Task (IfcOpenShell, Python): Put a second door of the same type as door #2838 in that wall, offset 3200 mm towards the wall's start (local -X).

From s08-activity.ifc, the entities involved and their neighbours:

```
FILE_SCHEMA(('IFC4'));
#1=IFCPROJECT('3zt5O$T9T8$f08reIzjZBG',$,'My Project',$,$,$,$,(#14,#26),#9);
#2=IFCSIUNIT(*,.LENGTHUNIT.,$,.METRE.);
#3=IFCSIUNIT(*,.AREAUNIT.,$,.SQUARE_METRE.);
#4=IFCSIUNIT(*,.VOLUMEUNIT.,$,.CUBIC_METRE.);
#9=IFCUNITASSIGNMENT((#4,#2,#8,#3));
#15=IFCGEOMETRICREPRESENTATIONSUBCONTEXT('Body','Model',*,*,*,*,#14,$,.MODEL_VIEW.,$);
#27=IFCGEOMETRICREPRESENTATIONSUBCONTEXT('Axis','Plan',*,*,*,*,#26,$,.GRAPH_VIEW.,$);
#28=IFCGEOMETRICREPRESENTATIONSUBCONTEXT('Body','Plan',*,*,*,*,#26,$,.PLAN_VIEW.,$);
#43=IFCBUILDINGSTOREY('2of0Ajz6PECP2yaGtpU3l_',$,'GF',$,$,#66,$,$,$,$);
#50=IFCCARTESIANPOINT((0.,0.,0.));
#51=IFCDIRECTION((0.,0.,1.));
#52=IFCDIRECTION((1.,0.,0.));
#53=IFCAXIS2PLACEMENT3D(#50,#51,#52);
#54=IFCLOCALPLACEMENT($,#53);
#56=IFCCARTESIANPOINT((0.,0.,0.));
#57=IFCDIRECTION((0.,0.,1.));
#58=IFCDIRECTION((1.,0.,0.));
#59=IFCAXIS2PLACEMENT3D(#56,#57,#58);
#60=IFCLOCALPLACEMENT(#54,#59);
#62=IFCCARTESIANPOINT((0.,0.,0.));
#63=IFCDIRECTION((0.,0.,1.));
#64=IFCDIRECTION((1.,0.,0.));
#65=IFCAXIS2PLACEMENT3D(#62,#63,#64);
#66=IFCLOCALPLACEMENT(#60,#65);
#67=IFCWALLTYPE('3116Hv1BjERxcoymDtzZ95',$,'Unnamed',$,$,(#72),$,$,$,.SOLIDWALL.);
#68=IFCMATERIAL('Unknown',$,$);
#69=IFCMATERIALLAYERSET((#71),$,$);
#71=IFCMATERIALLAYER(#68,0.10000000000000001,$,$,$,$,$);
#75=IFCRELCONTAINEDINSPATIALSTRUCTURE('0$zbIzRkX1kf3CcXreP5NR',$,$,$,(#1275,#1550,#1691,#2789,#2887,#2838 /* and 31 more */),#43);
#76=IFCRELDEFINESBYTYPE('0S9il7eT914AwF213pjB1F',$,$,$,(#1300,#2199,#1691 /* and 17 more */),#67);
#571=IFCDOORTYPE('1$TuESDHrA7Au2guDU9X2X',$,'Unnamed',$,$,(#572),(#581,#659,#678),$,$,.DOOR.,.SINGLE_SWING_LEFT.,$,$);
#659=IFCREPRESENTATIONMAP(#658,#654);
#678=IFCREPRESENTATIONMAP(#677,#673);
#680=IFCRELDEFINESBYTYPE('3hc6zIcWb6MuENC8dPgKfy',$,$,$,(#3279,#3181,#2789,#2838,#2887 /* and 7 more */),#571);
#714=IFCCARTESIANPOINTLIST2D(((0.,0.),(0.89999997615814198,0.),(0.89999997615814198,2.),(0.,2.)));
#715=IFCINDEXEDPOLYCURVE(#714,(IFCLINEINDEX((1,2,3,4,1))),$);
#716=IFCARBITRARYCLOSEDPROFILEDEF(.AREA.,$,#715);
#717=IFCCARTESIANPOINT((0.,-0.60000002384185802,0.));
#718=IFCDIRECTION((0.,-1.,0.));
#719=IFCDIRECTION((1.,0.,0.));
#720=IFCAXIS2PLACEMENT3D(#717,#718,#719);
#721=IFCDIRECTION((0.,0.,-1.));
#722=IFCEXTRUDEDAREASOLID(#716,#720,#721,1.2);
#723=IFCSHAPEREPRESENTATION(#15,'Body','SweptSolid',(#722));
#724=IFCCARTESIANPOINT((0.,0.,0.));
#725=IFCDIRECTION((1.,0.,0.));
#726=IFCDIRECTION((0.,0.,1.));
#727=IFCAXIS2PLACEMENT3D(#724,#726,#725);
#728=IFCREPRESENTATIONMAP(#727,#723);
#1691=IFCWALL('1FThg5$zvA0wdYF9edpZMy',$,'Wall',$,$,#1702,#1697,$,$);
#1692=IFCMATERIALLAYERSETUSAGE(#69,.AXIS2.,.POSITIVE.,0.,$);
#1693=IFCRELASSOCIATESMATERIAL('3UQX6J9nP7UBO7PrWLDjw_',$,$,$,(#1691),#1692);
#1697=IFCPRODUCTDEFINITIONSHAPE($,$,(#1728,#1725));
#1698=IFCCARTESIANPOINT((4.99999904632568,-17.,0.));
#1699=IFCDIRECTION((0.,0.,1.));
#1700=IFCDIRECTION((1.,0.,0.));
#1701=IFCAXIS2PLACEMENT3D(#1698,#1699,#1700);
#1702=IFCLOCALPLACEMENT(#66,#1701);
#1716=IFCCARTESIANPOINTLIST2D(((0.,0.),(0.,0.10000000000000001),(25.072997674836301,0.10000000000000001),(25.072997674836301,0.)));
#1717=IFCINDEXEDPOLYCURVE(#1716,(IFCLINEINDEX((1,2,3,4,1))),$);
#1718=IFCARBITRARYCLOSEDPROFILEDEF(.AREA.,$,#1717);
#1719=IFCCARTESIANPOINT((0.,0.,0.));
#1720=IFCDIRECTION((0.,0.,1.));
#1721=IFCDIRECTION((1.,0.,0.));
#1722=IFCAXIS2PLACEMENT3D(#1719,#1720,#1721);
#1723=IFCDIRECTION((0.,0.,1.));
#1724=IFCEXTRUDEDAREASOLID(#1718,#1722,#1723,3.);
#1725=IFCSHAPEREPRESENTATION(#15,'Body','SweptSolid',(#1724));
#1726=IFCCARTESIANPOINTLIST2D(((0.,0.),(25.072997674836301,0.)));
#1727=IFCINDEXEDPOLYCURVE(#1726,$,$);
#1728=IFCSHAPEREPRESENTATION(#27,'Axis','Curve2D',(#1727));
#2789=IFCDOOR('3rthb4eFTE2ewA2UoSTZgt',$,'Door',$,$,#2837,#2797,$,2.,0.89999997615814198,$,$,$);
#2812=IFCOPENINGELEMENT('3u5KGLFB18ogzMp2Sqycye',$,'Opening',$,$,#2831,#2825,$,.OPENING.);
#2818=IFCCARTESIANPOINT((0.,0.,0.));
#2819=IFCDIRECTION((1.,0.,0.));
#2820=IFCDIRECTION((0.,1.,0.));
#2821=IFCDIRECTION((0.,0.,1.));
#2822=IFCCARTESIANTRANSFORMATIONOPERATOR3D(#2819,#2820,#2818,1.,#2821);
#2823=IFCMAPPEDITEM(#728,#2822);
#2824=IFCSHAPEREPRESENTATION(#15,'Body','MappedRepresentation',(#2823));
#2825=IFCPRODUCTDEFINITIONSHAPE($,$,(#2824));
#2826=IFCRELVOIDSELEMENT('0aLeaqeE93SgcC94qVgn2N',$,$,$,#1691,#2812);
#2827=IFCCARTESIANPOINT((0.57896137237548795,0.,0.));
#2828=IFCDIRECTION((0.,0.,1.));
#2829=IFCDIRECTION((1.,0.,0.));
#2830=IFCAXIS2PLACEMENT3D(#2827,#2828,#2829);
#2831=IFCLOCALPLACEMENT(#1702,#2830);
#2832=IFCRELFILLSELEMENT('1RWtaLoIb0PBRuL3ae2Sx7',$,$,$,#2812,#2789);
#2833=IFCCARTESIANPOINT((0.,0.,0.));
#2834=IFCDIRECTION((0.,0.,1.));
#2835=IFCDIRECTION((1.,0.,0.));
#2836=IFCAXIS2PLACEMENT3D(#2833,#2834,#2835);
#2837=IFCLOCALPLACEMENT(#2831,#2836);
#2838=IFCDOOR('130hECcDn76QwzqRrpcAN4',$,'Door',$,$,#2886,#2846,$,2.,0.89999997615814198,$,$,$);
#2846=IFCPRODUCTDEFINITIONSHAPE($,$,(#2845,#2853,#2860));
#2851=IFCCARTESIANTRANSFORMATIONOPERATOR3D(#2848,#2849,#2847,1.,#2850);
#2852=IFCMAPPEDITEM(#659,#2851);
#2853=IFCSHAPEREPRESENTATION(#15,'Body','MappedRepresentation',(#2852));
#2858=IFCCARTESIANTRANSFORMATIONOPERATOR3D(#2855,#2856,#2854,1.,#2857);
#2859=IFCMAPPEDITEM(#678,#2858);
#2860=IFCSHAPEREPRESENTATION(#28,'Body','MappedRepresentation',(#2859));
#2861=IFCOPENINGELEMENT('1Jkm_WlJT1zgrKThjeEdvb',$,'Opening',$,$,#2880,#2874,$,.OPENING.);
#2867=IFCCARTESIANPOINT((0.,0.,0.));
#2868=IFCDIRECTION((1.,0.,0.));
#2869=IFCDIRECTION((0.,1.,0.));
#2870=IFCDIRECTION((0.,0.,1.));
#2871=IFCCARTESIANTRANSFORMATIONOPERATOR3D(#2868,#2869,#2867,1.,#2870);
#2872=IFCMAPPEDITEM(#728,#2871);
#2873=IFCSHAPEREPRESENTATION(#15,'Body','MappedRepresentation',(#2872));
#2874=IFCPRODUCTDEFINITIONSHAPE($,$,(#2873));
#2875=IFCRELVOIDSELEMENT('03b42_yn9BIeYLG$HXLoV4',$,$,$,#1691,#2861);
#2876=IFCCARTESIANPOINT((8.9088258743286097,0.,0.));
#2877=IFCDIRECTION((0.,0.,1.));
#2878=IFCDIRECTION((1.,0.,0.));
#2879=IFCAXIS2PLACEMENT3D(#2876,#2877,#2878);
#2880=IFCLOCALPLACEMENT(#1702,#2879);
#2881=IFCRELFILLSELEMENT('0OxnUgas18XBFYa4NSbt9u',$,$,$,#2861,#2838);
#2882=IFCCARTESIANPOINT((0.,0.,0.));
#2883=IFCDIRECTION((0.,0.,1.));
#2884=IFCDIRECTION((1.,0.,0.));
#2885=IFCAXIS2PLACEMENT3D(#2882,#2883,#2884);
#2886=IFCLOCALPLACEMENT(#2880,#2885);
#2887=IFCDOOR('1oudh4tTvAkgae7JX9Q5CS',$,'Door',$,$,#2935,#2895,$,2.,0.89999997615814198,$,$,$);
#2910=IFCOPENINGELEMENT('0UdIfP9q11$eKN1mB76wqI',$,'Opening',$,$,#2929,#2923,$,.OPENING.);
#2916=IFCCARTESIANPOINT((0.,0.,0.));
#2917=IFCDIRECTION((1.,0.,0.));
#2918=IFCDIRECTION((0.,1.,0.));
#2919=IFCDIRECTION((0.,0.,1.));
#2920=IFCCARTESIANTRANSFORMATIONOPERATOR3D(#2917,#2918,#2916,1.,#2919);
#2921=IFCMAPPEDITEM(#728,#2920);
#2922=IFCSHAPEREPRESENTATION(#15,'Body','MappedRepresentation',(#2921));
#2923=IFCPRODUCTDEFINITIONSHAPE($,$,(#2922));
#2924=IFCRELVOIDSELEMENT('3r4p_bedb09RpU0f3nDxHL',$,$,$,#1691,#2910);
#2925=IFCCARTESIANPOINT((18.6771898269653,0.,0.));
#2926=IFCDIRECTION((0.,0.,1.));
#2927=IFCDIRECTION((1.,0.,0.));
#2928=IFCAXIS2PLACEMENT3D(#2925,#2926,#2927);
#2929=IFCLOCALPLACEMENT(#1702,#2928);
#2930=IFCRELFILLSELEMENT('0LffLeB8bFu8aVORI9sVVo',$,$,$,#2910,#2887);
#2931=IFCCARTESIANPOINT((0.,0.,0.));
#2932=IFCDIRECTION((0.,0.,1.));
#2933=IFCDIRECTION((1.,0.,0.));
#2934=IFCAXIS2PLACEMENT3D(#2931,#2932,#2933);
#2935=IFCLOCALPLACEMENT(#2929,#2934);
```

```python
import ifcopenshell
import ifcopenshell.api.feature
import ifcopenshell.api.geometry
import ifcopenshell.api.root
import ifcopenshell.geom
import ifcopenshell.util.element
import ifcopenshell.util.placement
import ifcopenshell.util.shape
import ifcopenshell.util.unit

model = ifcopenshell.open("s08-activity.ifc")
unit_scale = ifcopenshell.util.unit.calculate_unit_scale(model)
settings = ifcopenshell.geom.settings()


def volume(element):
    """Net volume in cubic metres, openings subtracted."""
    shape = ifcopenshell.geom.create_shape(settings, element)
    return ifcopenshell.util.shape.get_volume(shape.geometry)


door = model.by_guid("130hECcDn76QwzqRrpcAN4")
opening = door.FillsVoids[0].RelatingOpeningElement
wall = opening.VoidsElements[0].RelatingBuildingElement
before = volume(wall)
shift = ifcopenshell.util.placement.get_local_placement(wall.ObjectPlacement)[:3, 0] * -3.2 / unit_scale

# copy_class copies the void relationship, type, container and properties, but no geometry.
new_opening = ifcopenshell.api.root.copy_class(model, product=opening)
new_opening.Representation = ifcopenshell.util.element.copy_deep(
    model, opening.Representation, exclude=["IfcGeometricRepresentationContext", "IfcRepresentationMap"]
)
new_door = ifcopenshell.api.root.copy_class(model, product=door)
new_door.Representation = ifcopenshell.util.element.copy_deep(
    model, door.Representation, exclude=["IfcGeometricRepresentationContext", "IfcRepresentationMap"]
)
ifcopenshell.api.feature.add_filling(model, opening=new_opening, element=new_door)

for old, new in ((opening, new_opening), (door, new_door)):
    matrix = ifcopenshell.util.placement.get_local_placement(old.ObjectPlacement)
    matrix[:3, 3] += shift
    ifcopenshell.api.geometry.edit_object_placement(model, product=new, matrix=matrix, is_si=False)

after = volume(wall)

print(f"wall volume {before:.3f} -> {after:.3f} m3")

model.write("s08-activity-out.ifc")
```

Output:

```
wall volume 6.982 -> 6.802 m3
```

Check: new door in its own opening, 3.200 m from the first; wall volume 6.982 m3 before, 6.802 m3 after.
